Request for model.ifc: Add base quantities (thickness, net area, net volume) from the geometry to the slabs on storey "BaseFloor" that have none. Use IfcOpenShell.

First a look at what the model holds.

```python
import ifcopenshell
import ifcopenshell.util.element
import ifcopenshell.util.unit

model = ifcopenshell.open("model.ifc")
print(model.schema)
for unit_type in ("LENGTHUNIT", "AREAUNIT", "VOLUMEUNIT"):
    print(unit_type, ifcopenshell.util.unit.calculate_unit_scale(model, unit_type))
storey = next(s for s in model.by_type("IfcBuildingStorey") if s.Name == "BaseFloor")
slabs = [e for e in ifcopenshell.util.element.get_decomposition(storey) if e.is_a("IfcSlab")]
for e in sorted(slabs, key=lambda e: e.id()):
    print(e.id(), e.is_a(), e.Name, list(ifcopenshell.util.element.get_psets(e, qtos_only=True)), sep=" | ")
```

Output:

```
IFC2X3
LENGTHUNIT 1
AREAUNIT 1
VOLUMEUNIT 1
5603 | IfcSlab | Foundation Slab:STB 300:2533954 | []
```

```python
import ifcopenshell
import ifcopenshell.api.pset
import ifcopenshell.geom
import ifcopenshell.util.element
import ifcopenshell.util.shape
import ifcopenshell.util.unit

model = ifcopenshell.open("model.ifc")
unit_scale = ifcopenshell.util.unit.calculate_unit_scale(model)
area_scale = ifcopenshell.util.unit.calculate_unit_scale(model, "AREAUNIT")
volume_scale = ifcopenshell.util.unit.calculate_unit_scale(model, "VOLUMEUNIT")
settings = ifcopenshell.geom.settings()

storey = next(s for s in model.by_type("IfcBuildingStorey") if s.Name == "BaseFloor")
slabs = [e for e in ifcopenshell.util.element.get_decomposition(storey) if e.is_a("IfcSlab")]

for e in sorted(slabs, key=lambda e: e.id()):
    if ifcopenshell.util.element.get_psets(e, qtos_only=True, should_inherit=False):
        continue
    # Geometry comes back in metres, in the element's own axes.
    shape = ifcopenshell.geom.create_shape(settings, e)
    values = {
        "Width": ifcopenshell.util.shape.get_z(shape.geometry) / unit_scale,
        "NetArea": ifcopenshell.util.shape.get_footprint_area(shape.geometry) / area_scale,
        "NetVolume": ifcopenshell.util.shape.get_volume(shape.geometry) / volume_scale,
    }
    qto = ifcopenshell.api.pset.add_qto(model, product=e, name="BaseQuantities")
    ifcopenshell.api.pset.edit_qto(model, qto=qto, properties=values)
    print(e.id(), {k: round(v, 3) for k, v in values.items()})

model.write("model_rev.ifc")
```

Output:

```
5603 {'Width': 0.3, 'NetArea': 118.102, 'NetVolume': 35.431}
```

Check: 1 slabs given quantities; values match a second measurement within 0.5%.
